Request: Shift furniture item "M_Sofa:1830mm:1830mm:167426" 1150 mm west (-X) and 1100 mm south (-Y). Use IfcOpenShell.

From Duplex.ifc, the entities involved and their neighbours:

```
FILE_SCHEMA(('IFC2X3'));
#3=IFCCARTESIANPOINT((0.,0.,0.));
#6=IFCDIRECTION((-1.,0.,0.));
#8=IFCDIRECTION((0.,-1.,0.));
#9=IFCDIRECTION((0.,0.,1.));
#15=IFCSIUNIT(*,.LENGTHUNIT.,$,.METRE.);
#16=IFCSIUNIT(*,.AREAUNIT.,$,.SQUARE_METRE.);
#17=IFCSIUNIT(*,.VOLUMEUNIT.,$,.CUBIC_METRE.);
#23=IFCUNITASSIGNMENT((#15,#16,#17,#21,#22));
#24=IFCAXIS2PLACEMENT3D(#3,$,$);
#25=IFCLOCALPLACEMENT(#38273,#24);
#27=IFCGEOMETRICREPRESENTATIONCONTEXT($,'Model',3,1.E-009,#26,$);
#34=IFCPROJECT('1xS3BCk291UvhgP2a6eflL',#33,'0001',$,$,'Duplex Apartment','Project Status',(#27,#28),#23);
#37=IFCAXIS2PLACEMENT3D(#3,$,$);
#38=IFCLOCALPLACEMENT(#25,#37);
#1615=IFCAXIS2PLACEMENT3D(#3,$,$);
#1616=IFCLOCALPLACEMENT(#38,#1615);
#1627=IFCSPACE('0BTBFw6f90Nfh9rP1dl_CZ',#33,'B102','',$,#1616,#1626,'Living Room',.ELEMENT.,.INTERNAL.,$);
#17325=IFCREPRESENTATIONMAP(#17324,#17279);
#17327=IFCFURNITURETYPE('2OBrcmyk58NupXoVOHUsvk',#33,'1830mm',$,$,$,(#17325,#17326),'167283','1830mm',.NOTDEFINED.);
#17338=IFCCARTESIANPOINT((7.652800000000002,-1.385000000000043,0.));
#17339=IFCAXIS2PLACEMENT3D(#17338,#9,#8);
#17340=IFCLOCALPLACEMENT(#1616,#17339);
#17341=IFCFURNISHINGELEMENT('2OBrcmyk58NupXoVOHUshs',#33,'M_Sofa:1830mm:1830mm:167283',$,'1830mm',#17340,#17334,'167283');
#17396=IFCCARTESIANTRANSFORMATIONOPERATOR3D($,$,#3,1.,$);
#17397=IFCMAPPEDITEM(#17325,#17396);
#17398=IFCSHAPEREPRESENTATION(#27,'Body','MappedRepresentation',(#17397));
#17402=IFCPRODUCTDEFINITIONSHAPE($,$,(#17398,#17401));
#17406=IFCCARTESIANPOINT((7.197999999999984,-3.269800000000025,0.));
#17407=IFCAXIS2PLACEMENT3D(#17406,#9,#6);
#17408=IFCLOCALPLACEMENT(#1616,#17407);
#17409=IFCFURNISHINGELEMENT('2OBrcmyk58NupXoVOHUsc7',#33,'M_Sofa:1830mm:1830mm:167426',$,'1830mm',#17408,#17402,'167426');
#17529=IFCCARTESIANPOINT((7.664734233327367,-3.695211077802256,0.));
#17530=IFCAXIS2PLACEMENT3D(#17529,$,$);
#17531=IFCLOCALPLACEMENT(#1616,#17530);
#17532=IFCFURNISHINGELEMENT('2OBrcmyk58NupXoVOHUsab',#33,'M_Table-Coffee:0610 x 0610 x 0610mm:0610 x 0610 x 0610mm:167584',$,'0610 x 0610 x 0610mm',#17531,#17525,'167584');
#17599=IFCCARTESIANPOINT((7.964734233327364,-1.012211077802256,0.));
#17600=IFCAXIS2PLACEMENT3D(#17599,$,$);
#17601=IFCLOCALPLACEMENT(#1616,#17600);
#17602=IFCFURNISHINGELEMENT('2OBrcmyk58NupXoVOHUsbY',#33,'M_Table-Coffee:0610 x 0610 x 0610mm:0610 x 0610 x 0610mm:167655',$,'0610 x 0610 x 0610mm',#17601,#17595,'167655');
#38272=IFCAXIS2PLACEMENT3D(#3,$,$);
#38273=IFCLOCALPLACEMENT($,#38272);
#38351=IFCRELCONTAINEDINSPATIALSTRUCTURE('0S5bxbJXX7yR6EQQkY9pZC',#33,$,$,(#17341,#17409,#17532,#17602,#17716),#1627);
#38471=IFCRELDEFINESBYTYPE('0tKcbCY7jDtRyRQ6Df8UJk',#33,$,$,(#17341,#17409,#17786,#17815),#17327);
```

```python
import ifcopenshell
import ifcopenshell.api.geometry
import ifcopenshell.util.placement
import ifcopenshell.util.unit

model = ifcopenshell.open("Duplex.ifc")
unit_scale = ifcopenshell.util.unit.calculate_unit_scale(model)

item = model.by_id(17409)
matrix = ifcopenshell.util.placement.get_local_placement(item.ObjectPlacement)
matrix[0, 3] -= 1.15 / unit_scale
matrix[1, 3] -= 1.1 / unit_scale
ifcopenshell.api.geometry.edit_object_placement(model, product=item, matrix=matrix, is_si=False)

print(ifcopenshell.util.placement.get_local_placement(item.ObjectPlacement).round(3) + 0.0)

model.write("Duplex_v2.ifc")
```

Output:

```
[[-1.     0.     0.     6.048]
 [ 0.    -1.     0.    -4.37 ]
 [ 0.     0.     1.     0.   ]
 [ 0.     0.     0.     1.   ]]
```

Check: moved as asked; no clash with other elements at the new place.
